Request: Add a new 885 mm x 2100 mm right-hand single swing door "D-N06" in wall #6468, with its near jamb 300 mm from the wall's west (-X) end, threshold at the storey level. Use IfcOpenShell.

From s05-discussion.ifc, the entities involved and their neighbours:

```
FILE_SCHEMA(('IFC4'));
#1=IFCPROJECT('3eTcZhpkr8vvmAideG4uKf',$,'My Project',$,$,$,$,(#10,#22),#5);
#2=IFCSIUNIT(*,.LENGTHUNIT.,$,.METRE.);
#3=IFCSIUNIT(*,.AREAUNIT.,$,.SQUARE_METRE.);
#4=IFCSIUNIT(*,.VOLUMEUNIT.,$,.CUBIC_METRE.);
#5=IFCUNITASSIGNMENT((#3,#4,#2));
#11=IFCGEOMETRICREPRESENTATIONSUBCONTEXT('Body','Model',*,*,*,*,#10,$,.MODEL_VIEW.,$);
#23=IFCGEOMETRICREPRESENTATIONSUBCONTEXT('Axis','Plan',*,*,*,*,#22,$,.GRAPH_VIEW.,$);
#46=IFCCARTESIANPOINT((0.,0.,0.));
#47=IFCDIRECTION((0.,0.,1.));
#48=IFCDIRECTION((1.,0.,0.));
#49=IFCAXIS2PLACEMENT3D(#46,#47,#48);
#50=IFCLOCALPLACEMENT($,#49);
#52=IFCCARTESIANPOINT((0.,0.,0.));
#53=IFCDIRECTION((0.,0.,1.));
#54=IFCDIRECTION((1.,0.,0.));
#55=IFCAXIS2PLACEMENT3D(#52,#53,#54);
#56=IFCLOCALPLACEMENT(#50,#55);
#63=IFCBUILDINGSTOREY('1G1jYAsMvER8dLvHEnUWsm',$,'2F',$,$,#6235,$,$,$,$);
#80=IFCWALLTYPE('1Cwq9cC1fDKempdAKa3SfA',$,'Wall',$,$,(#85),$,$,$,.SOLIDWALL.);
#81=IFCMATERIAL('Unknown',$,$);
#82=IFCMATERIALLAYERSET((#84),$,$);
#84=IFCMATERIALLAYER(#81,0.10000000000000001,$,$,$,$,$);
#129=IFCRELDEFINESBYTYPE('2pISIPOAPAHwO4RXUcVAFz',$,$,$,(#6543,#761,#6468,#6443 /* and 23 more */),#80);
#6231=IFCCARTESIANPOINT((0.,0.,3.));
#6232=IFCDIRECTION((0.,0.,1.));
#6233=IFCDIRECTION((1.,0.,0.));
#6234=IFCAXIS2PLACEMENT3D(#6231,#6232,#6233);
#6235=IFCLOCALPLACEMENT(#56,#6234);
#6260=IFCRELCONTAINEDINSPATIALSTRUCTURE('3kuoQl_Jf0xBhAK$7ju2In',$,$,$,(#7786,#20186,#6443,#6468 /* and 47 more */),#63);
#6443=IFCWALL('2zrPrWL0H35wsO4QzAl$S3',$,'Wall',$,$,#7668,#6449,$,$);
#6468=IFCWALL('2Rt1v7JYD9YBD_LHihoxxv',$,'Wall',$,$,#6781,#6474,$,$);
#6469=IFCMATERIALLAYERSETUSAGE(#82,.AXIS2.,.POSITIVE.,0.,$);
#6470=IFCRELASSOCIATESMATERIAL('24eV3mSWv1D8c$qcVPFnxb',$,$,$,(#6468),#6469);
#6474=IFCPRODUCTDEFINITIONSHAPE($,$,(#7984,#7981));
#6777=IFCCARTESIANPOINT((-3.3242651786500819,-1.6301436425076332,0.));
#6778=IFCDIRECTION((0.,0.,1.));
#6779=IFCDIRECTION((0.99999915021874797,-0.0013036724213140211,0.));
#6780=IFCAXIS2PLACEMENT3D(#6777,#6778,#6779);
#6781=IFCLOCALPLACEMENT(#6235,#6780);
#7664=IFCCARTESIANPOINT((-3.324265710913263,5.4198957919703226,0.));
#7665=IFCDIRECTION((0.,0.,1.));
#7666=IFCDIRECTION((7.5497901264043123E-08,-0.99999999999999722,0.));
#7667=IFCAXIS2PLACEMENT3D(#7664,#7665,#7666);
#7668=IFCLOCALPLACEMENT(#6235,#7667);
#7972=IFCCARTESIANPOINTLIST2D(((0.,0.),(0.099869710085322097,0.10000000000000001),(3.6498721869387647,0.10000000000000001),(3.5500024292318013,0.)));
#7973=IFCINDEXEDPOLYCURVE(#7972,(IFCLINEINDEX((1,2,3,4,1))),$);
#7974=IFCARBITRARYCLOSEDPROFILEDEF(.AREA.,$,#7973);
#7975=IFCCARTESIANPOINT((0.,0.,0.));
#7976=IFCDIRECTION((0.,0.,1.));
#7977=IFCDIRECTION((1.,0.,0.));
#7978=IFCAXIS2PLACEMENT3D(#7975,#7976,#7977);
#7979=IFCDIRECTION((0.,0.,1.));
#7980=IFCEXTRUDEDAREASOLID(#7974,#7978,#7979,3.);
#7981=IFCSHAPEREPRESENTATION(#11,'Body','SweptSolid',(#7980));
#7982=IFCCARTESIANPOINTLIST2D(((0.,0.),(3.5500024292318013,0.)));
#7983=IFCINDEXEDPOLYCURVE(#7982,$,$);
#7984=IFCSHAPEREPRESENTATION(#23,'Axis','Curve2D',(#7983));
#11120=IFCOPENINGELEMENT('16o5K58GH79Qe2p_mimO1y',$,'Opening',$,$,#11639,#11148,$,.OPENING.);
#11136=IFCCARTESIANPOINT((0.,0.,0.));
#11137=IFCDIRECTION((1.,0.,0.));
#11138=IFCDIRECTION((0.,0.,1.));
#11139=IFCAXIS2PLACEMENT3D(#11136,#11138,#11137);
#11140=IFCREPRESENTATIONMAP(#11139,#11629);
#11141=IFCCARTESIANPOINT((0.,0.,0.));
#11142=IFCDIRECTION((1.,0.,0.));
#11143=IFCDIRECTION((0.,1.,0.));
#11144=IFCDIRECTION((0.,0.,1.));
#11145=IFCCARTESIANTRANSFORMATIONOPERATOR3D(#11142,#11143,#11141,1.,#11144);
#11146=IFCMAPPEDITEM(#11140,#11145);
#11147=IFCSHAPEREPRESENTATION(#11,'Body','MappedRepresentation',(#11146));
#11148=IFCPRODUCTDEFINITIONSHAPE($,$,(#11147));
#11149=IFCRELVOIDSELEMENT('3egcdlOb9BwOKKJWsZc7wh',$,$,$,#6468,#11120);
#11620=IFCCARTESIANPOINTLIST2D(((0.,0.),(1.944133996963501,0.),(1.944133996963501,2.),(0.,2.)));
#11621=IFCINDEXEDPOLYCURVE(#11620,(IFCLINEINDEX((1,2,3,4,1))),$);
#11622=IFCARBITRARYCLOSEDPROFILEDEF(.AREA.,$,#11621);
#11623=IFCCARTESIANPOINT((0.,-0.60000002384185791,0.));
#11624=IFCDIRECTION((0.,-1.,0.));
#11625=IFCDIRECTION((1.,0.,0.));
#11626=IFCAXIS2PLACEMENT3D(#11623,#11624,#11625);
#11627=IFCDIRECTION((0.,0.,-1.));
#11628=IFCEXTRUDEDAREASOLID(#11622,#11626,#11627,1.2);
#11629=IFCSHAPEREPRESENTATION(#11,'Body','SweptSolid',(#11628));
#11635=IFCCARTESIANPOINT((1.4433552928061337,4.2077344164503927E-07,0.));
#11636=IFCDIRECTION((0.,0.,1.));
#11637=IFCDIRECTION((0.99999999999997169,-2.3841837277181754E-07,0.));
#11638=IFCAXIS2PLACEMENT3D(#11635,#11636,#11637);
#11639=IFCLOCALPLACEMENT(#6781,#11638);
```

```python
import numpy as np
import ifcopenshell
import ifcopenshell.api.feature
import ifcopenshell.api.geometry
import ifcopenshell.api.root
import ifcopenshell.api.spatial
import ifcopenshell.geom
import ifcopenshell.util.element
import ifcopenshell.util.placement
import ifcopenshell.util.representation
import ifcopenshell.util.shape
import ifcopenshell.util.unit

model = ifcopenshell.open("s05-discussion.ifc")
unit_scale = ifcopenshell.util.unit.calculate_unit_scale(model)
settings = ifcopenshell.geom.settings()


def volume(element):
    """Net volume in cubic metres, openings subtracted."""
    shape = ifcopenshell.geom.create_shape(settings, element)
    return ifcopenshell.util.shape.get_volume(shape.geometry)


wall = model.by_id(6468)
storey = ifcopenshell.util.element.get_container(wall, ifc_class="IfcBuildingStorey")
context = ifcopenshell.util.representation.get_context(model, "Model", "Body", "MODEL_VIEW")
before = volume(wall)

width, height, from_end, sill = 0.885, 2.1, 0.3, 0.0  # metres

# The wall runs along its own X axis, and the end named is its -X end.
wall_shape = ifcopenshell.geom.create_shape(settings, wall)
x, y, z = ifcopenshell.util.shape.get_vertices(wall_shape.geometry).T
start = x.min() + from_end
face, thickness = float(y.min()), float(y.max() - y.min())
wall_matrix = ifcopenshell.util.placement.get_local_placement(wall.ObjectPlacement)
level = ifcopenshell.util.placement.get_local_placement(storey.ObjectPlacement)[2, 3]


def in_wall(x, y):
    """Placement at x, y metres in the wall's axes, at sill height."""
    matrix = wall_matrix.copy()
    matrix[:, 3] = wall_matrix @ np.array([x / unit_scale, y / unit_scale, 0.0, 1.0])
    matrix[2, 3] = level + sill / unit_scale
    return matrix


# Opening: a box that overshoots both wall faces by 50 mm.
opening = ifcopenshell.api.root.create_entity(model, ifc_class="IfcOpeningElement", predefined_type="OPENING")
box = ifcopenshell.api.geometry.add_wall_representation(
    model, context=context, length=width, height=height, thickness=thickness + 0.1
)
ifcopenshell.api.geometry.assign_representation(model, product=opening, representation=box)
ifcopenshell.api.geometry.edit_object_placement(model, product=opening, matrix=in_wall(start, face - 0.05), is_si=False)
ifcopenshell.api.feature.add_feature(model, feature=opening, element=wall)

door = ifcopenshell.api.root.create_entity(model, ifc_class="IfcDoor", name="D-N06", predefined_type="DOOR")
door.OverallWidth, door.OverallHeight = width / unit_scale, height / unit_scale
door.OperationType = "SINGLE_SWING_RIGHT"
body = ifcopenshell.api.geometry.add_door_representation(
    model,
    context=context,
    overall_width=door.OverallWidth,
    overall_height=door.OverallHeight,
    operation_type="SINGLE_SWING_RIGHT",
    lining_properties={"LiningDepth": thickness / unit_scale, "ThresholdDepth": thickness / unit_scale},
)
ifcopenshell.api.geometry.assign_representation(model, product=door, representation=body)
ifcopenshell.api.spatial.assign_container(model, products=[door], relating_structure=storey)
ifcopenshell.api.feature.add_filling(model, opening=opening, element=door)

# The lining spans the wall, so the door starts at the wall face.
ifcopenshell.api.geometry.edit_object_placement(model, product=door, matrix=in_wall(start, face), is_si=False)

after = volume(wall)

print(f"wall volume {before:.3f} -> {after:.3f} m3")

model.write("s05-discussion_v2.ifc")
```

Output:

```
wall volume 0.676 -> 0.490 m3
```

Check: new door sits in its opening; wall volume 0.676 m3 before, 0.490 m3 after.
